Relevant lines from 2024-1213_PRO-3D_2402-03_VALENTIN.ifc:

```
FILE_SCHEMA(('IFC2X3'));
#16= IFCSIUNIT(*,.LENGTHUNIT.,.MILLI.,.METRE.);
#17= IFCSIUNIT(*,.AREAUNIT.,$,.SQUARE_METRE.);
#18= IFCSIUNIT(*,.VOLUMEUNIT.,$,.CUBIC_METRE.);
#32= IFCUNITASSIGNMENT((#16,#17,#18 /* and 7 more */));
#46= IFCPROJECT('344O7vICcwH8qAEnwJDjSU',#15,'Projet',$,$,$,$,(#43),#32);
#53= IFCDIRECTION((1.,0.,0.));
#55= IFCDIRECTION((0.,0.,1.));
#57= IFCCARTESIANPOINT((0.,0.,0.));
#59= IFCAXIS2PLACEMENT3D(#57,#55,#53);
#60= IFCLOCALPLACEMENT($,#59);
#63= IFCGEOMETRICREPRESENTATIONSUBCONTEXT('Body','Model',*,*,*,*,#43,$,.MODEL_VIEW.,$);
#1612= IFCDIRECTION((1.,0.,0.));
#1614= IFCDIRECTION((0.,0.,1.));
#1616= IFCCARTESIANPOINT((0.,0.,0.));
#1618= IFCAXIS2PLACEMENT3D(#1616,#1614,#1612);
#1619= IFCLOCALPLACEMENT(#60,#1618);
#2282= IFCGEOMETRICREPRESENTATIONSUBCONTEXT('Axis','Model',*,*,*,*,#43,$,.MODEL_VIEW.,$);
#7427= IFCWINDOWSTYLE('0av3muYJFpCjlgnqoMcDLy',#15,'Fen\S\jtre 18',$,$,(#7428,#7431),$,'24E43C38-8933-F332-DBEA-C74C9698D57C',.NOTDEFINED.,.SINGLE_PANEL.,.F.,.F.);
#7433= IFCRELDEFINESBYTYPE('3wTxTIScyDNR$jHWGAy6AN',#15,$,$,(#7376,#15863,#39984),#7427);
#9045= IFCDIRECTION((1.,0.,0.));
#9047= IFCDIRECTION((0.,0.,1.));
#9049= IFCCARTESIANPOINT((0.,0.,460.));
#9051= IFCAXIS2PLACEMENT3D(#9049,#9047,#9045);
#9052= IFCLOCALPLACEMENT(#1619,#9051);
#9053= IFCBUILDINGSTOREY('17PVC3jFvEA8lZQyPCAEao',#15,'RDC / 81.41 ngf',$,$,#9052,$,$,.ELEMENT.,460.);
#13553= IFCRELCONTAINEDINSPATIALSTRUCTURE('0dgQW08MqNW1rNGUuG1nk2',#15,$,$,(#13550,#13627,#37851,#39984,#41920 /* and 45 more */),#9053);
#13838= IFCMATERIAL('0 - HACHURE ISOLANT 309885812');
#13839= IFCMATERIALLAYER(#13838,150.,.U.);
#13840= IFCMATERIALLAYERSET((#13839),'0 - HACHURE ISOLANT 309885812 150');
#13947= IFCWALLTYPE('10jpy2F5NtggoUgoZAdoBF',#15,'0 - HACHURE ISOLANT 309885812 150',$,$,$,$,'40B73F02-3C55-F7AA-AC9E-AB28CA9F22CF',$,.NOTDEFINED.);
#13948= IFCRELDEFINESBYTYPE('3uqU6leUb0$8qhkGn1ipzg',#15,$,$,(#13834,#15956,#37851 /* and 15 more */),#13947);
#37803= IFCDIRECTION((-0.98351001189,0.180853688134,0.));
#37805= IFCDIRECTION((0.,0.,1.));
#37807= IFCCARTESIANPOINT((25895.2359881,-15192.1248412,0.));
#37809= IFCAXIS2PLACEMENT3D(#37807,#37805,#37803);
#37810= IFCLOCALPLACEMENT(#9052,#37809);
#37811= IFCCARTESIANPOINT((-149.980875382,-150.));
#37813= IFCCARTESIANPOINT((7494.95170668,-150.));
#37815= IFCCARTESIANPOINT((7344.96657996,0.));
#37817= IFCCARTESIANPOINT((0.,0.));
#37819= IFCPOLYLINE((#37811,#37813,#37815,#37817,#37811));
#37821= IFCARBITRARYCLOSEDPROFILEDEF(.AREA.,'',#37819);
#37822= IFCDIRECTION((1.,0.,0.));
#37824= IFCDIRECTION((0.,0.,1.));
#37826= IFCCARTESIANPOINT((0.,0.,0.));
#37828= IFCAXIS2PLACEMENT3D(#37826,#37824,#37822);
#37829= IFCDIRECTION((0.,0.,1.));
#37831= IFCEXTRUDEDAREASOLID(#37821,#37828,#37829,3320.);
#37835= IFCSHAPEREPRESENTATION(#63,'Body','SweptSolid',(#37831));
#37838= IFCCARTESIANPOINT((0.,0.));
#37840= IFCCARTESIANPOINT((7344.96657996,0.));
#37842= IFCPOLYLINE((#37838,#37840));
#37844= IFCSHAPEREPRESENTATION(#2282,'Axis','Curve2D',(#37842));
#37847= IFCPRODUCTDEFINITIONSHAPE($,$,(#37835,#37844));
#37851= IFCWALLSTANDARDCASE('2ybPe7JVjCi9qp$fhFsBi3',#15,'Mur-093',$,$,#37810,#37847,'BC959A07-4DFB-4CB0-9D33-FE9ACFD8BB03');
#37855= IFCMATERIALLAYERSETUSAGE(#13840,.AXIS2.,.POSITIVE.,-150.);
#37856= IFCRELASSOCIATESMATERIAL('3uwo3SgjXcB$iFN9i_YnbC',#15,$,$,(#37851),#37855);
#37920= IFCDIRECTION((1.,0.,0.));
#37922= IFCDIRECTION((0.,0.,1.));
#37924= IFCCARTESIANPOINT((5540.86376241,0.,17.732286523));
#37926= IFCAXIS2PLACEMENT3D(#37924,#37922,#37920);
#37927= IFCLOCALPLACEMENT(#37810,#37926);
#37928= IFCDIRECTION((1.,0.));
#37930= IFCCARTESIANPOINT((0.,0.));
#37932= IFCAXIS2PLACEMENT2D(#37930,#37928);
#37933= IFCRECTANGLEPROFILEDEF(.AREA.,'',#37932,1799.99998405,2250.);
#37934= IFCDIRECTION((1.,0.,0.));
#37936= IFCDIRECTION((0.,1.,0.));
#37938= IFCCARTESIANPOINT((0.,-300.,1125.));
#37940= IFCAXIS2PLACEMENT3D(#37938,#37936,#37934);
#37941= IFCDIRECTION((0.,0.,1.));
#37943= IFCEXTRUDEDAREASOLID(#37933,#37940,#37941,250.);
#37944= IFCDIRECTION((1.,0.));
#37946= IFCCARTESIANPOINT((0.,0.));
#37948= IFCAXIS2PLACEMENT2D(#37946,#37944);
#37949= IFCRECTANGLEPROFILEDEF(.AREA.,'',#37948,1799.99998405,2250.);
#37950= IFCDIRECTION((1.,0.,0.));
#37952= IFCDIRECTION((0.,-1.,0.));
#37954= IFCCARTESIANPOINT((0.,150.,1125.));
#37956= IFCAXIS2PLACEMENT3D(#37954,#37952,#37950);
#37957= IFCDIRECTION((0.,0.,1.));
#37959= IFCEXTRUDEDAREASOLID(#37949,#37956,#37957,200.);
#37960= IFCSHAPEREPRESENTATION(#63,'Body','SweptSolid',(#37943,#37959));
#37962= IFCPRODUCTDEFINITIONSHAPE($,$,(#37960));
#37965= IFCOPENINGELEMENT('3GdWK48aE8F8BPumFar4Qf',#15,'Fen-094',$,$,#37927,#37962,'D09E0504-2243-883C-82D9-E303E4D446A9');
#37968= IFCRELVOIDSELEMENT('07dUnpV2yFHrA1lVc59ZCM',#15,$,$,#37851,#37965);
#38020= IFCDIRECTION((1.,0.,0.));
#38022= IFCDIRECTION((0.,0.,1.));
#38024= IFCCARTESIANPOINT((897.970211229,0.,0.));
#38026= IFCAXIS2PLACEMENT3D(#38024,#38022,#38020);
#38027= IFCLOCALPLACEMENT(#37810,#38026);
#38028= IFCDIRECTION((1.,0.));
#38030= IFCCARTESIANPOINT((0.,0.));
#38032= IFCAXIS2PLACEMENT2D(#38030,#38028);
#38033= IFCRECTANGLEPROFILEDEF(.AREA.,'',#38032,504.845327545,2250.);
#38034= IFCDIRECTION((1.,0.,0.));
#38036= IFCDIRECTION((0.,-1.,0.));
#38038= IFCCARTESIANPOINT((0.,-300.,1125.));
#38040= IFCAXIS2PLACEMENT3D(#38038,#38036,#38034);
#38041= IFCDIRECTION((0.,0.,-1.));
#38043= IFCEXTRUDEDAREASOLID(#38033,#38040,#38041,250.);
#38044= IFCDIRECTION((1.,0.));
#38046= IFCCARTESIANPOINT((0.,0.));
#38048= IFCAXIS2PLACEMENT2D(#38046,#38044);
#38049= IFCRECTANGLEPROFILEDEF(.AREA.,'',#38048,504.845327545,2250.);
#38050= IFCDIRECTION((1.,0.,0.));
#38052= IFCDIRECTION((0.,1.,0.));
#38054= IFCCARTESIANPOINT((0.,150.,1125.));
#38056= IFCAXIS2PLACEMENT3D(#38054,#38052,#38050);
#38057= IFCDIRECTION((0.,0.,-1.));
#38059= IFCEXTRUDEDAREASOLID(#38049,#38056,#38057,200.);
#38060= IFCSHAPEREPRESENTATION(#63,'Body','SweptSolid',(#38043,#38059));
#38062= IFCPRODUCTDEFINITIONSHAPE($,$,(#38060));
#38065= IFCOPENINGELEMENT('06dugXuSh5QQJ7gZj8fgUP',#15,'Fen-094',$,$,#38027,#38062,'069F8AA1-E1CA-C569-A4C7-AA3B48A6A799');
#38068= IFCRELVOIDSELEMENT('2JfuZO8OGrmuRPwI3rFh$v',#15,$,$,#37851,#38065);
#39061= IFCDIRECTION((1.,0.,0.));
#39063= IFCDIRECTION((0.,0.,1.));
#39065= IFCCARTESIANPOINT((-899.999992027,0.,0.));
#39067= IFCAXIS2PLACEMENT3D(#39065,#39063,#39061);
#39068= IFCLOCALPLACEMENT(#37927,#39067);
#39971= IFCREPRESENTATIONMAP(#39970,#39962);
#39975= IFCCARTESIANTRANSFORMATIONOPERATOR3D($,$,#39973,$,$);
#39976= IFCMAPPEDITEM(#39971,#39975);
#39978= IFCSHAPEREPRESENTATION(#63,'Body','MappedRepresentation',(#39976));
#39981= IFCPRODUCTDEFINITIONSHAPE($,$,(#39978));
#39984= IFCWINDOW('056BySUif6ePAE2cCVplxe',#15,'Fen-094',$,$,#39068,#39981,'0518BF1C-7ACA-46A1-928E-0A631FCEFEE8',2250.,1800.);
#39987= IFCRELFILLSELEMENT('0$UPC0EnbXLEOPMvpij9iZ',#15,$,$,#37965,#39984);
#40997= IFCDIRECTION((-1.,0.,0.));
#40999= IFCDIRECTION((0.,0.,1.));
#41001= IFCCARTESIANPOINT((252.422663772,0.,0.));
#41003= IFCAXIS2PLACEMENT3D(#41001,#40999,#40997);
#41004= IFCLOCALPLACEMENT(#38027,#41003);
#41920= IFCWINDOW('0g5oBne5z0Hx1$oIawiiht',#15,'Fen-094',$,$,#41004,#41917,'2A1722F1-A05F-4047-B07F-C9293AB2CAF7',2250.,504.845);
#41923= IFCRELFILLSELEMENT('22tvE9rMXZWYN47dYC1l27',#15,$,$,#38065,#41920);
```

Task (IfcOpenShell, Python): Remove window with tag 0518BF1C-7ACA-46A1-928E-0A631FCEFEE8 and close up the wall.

```python
import ifcopenshell
import ifcopenshell.api.feature
import ifcopenshell.api.root
import ifcopenshell.geom
import ifcopenshell.util.shape

model = ifcopenshell.open("2024-1213_PRO-3D_2402-03_VALENTIN.ifc")
settings = ifcopenshell.geom.settings()


def volume(element):
    """Net volume in cubic metres, openings subtracted."""
    shape = ifcopenshell.geom.create_shape(settings, element)
    return ifcopenshell.util.shape.get_volume(shape.geometry)


window = model.by_id(39984)
opening = window.FillsVoids[0].RelatingOpeningElement
wall = opening.VoidsElements[0].RelatingBuildingElement
before = volume(wall)

ifcopenshell.api.root.remove_product(model, product=window)
ifcopenshell.api.feature.remove_feature(model, feature=opening)

after = volume(wall)

print(f"wall volume {before:.3f} -> {after:.3f} m3")

model.write("2024-1213_PRO-3D_2402-03_VALENTIN_updated.ifc")
```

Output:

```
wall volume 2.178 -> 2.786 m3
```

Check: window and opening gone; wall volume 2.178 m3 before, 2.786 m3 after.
